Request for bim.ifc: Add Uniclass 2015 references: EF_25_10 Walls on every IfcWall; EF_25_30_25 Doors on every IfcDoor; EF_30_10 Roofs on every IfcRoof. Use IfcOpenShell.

First a look at what the model holds.

```python
import ifcopenshell

model = ifcopenshell.open("bim.ifc")
print(model.schema)
print("classifications:", [c.Name for c in model.by_type("IfcClassification")])
for ifc_class in ("IfcDoor", "IfcRoof", "IfcStair", "IfcWall", "IfcWindow"):
    print(ifc_class, len(model.by_type(ifc_class)))
```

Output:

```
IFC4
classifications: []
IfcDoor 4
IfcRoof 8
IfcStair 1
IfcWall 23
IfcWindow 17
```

```python
import ifcopenshell
import ifcopenshell.api.classification

model = ifcopenshell.open("bim.ifc")

system = ifcopenshell.api.classification.add_classification(model, classification="Uniclass 2015")

codes = {
    "IfcWall": ("EF_25_10", "Walls"),
    "IfcDoor": ("EF_25_30_25", "Doors"),
    "IfcRoof": ("EF_30_10", "Roofs"),
}
for ifc_class, (code, name) in codes.items():
    products = model.by_type(ifc_class)
    ifcopenshell.api.classification.add_reference(
        model, products=products, classification=system, identification=code, name=name
    )
    print(code, len(products))

model.write("bim-out.ifc")
```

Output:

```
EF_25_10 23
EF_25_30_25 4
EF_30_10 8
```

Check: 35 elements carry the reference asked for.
